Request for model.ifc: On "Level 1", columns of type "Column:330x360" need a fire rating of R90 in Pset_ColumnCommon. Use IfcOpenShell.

First a look at what the model holds.

```python
import ifcopenshell
import ifcopenshell.util.element

model = ifcopenshell.open("model.ifc")
print(model.schema)
storey = next(s for s in model.by_type("IfcBuildingStorey") if s.Name == "Level 1")
columns = [e for e in ifcopenshell.util.element.get_decomposition(storey) if e.is_a("IfcColumn")]
seen = {}
for e in columns:
    element_type = ifcopenshell.util.element.get_type(e)
    key = (element_type.Name if element_type != e and element_type else None, ifcopenshell.util.element.get_pset(e, "Pset_ColumnCommon", "FireRating"))
    seen[key] = seen.get(key, 0) + 1
for (name, value), count in sorted(seen.items(), key=str):
    print(count, "x", name, "|", value)
```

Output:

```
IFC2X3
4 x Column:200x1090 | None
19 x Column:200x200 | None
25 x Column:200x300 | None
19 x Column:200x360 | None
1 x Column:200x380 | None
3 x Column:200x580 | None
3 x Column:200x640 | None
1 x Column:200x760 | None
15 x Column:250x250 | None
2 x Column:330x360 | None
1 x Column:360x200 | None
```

```python
import ifcopenshell
import ifcopenshell.api.pset
import ifcopenshell.util.element

model = ifcopenshell.open("model.ifc")

storey = next(s for s in model.by_type("IfcBuildingStorey") if s.Name == "Level 1")
columns = [e for e in ifcopenshell.util.element.get_decomposition(storey) if e.is_a("IfcColumn")]

count = 0
for e in columns:
    element_type = ifcopenshell.util.element.get_type(e)
    if element_type in (None, e) or element_type.Name != "Column:330x360":
        continue
    # add_pset returns the element's existing set when there is one.
    pset = ifcopenshell.api.pset.add_pset(model, product=e, name="Pset_ColumnCommon")
    ifcopenshell.api.pset.edit_pset(model, pset=pset, properties={"FireRating": "R90"})
    count += 1

print(count, "columns updated")

model.write("model_edited.ifc")
```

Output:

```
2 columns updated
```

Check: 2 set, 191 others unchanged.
